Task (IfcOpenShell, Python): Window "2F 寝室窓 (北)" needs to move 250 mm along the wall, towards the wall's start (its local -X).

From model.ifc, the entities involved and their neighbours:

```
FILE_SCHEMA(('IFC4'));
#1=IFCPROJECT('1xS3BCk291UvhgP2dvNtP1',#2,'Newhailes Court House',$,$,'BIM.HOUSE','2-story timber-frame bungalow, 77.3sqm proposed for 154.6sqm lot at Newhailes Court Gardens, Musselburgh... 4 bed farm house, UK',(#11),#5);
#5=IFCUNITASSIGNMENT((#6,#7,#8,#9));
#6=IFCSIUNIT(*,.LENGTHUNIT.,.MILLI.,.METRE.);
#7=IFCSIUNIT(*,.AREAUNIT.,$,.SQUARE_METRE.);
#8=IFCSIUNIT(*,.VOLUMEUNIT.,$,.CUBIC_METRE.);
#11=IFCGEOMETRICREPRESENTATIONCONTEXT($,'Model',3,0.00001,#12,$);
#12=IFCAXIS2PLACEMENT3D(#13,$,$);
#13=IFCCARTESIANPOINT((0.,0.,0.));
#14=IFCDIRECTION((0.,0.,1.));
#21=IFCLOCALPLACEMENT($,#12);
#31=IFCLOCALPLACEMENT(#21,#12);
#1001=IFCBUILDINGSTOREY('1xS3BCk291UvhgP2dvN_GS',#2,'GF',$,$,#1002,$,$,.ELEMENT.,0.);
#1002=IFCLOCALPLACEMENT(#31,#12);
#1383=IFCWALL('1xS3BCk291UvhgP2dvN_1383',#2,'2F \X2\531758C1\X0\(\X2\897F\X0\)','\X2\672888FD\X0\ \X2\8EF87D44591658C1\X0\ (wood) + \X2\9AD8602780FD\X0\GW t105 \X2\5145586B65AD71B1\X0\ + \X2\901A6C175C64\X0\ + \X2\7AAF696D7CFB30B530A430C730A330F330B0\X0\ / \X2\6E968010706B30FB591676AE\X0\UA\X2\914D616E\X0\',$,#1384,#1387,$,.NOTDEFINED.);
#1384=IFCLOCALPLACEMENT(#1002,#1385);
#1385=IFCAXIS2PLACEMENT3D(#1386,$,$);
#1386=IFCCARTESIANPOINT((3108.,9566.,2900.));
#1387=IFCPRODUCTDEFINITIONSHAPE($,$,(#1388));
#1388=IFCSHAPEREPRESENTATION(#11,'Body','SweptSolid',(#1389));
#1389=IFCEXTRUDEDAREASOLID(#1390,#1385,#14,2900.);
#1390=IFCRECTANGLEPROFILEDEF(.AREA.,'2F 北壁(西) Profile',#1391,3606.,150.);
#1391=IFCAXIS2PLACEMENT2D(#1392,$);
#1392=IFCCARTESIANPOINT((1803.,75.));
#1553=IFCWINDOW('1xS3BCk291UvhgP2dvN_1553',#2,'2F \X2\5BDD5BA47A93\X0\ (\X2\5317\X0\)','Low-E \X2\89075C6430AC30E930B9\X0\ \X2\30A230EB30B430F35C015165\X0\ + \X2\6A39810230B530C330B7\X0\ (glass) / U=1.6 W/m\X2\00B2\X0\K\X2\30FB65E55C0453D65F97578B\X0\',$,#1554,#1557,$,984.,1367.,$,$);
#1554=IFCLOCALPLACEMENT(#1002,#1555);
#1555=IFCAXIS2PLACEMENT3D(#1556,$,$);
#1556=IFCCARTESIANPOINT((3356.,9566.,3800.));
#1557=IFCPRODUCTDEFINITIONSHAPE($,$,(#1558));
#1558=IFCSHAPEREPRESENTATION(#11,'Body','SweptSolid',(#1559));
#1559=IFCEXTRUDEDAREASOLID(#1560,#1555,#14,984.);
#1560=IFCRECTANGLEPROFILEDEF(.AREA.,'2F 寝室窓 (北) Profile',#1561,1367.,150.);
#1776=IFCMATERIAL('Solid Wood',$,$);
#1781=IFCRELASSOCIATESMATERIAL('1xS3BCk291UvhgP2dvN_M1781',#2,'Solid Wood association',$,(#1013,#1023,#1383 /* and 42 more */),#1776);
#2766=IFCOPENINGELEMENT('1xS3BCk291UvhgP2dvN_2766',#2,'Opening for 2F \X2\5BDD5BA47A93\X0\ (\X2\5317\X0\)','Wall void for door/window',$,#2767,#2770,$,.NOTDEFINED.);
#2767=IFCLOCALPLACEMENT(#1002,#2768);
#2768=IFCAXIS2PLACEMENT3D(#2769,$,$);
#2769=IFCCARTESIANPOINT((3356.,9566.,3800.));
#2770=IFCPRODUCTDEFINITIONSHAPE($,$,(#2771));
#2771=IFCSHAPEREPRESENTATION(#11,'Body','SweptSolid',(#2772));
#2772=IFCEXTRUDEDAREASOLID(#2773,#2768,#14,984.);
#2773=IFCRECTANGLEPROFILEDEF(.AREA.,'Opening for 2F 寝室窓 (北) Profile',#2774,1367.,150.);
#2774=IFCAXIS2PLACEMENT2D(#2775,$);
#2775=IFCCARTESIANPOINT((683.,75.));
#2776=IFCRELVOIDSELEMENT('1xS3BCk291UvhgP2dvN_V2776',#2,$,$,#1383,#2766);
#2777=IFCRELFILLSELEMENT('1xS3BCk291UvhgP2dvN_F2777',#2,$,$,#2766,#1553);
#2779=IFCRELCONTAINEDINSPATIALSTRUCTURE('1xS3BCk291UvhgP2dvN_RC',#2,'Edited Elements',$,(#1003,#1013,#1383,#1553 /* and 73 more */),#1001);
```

```python
import ifcopenshell
import ifcopenshell.api.geometry
import ifcopenshell.util.placement

model = ifcopenshell.open("model.ifc")

window = model.by_id(1553)
opening = window.FillsVoids[0].RelatingOpeningElement
wall = opening.VoidsElements[0].RelatingBuildingElement

wall_matrix = ifcopenshell.util.placement.get_local_placement(wall.ObjectPlacement)
shift = wall_matrix[:3, 0] * -250.0
before = ifcopenshell.util.placement.get_local_placement(window.ObjectPlacement)[:3, 3].copy()

# The window is not placed relative to its opening, so move both.
for product in (opening, window):
    matrix = ifcopenshell.util.placement.get_local_placement(product.ObjectPlacement)
    matrix[:3, 3] += shift
    ifcopenshell.api.geometry.edit_object_placement(model, product=product, matrix=matrix, is_si=False)

after = ifcopenshell.util.placement.get_local_placement(window.ObjectPlacement)[:3, 3]
print("window moved by", (after - before).round(3) + 0.0)

model.write("model_rev.ifc")
```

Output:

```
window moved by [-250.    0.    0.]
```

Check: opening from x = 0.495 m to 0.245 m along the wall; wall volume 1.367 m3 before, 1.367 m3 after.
